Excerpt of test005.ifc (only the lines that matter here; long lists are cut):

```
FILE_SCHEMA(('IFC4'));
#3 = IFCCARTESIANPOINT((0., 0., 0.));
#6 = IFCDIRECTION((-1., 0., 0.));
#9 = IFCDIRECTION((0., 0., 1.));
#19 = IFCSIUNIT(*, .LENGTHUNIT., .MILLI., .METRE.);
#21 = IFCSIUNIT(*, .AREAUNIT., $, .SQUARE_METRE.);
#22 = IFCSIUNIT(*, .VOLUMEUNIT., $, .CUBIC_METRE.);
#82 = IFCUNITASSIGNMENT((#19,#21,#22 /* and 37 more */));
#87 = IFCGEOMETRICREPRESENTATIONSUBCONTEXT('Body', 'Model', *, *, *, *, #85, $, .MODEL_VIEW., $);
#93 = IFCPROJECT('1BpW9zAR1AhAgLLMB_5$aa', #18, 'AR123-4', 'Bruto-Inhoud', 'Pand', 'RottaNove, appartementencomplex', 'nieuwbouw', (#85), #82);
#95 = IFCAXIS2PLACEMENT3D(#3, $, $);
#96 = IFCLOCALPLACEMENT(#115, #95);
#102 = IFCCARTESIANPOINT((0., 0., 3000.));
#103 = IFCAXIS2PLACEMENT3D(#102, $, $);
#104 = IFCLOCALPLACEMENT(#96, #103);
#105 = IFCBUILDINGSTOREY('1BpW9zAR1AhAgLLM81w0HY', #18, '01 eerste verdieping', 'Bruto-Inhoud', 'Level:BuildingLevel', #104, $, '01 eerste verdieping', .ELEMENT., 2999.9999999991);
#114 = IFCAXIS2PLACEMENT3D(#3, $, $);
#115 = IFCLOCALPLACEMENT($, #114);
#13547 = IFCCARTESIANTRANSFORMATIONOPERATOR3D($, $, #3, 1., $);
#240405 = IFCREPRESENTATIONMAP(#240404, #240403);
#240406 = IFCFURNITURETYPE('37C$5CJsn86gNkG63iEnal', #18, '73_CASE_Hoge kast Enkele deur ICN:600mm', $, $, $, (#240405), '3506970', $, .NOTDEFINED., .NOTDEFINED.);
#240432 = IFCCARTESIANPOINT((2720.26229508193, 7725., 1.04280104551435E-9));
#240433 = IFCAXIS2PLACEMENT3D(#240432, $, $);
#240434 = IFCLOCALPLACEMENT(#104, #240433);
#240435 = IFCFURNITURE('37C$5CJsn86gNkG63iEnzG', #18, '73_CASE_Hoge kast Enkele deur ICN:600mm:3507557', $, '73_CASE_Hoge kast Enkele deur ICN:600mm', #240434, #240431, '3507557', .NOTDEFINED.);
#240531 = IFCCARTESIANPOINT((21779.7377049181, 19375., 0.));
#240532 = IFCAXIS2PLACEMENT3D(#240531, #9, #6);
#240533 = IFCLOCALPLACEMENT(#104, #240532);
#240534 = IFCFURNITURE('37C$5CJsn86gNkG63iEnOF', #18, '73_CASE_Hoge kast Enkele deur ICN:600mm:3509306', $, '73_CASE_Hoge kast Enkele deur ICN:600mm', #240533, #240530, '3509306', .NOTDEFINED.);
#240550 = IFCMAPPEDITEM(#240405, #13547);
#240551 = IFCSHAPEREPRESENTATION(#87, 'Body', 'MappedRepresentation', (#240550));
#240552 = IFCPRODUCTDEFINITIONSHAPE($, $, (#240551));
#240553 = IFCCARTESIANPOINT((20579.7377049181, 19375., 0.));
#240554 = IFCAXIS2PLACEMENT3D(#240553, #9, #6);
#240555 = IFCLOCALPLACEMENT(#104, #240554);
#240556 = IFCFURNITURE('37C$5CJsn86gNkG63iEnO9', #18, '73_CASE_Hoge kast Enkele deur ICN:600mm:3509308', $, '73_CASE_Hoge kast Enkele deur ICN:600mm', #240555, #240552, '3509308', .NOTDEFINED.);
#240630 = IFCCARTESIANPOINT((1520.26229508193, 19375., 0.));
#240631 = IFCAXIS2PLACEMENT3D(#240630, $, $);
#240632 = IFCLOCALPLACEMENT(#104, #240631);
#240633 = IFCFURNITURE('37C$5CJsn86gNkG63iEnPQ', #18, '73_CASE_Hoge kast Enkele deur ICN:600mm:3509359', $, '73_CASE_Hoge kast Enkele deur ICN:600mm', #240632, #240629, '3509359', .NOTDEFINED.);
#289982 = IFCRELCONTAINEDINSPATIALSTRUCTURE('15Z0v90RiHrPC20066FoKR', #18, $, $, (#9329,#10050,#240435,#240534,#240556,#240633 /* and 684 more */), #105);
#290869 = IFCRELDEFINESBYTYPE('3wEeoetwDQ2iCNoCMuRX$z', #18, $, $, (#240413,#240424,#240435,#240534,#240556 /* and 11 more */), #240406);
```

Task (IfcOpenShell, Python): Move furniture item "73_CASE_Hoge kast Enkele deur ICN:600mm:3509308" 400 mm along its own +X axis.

```python
import ifcopenshell
import ifcopenshell.api.geometry
import ifcopenshell.util.placement
import ifcopenshell.util.unit

model = ifcopenshell.open("test005.ifc")
unit_scale = ifcopenshell.util.unit.calculate_unit_scale(model)

item = model.by_guid("37C$5CJsn86gNkG63iEnO9")
matrix = ifcopenshell.util.placement.get_local_placement(item.ObjectPlacement)
matrix[:3, 3] += matrix[:3, 0] * 0.4 / unit_scale
ifcopenshell.api.geometry.edit_object_placement(model, product=item, matrix=matrix, is_si=False)

print(ifcopenshell.util.placement.get_local_placement(item.ObjectPlacement).round(3) + 0.0)

model.write("test005_edited.ifc")
```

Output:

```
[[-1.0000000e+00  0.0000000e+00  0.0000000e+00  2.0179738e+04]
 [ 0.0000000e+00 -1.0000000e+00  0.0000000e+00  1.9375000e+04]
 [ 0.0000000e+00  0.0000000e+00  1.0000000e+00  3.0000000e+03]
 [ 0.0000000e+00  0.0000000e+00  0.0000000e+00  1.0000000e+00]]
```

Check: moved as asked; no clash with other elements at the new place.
